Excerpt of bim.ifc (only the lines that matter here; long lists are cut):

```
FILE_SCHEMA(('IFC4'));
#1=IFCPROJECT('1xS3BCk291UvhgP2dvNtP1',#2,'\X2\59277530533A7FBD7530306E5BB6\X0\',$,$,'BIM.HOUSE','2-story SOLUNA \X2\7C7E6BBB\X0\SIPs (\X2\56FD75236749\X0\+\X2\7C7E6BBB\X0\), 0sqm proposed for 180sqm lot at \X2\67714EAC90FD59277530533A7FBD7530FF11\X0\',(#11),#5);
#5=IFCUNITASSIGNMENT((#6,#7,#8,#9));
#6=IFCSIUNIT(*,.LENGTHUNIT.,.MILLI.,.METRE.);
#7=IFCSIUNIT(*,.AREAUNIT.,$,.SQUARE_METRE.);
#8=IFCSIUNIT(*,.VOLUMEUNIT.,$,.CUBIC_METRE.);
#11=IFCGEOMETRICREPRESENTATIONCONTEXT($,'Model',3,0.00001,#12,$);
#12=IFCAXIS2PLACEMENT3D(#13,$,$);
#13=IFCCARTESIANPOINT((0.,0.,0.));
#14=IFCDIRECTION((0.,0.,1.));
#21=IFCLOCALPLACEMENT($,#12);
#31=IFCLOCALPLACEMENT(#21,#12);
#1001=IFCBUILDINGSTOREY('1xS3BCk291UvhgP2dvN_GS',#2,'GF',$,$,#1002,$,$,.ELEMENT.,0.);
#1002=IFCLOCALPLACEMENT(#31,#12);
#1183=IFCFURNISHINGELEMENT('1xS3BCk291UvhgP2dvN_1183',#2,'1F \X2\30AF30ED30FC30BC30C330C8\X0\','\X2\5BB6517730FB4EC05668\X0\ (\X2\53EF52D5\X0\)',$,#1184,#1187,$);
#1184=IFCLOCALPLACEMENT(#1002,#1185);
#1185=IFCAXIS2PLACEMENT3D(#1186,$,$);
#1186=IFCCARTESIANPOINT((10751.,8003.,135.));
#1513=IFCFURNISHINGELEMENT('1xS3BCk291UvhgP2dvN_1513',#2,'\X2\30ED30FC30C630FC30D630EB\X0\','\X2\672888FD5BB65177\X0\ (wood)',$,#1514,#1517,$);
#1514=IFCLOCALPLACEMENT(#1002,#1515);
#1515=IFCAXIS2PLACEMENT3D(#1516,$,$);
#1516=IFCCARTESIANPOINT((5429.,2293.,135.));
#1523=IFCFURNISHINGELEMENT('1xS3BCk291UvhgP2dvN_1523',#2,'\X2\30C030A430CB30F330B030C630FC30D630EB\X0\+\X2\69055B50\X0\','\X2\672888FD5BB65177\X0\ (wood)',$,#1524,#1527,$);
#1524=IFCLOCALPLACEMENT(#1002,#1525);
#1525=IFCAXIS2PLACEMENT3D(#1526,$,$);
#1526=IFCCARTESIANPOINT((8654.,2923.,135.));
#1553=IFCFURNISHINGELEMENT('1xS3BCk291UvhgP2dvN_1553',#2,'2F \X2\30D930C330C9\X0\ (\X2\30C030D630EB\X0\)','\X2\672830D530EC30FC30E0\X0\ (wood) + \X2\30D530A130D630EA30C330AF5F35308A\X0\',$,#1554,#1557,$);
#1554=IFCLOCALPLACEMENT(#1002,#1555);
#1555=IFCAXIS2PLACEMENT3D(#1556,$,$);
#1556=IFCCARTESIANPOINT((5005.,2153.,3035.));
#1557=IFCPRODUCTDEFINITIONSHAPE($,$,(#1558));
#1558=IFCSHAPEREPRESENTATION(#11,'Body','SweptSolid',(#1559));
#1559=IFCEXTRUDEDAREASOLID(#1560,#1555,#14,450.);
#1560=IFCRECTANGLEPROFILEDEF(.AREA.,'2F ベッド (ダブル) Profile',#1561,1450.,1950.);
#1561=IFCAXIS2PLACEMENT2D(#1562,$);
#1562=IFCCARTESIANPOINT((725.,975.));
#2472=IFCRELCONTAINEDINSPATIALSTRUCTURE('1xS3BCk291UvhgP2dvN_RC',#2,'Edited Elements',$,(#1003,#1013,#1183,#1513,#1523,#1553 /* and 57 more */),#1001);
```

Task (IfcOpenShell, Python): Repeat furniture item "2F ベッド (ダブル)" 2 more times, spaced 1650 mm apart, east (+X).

```python
import numpy as np
import ifcopenshell
import ifcopenshell.api.geometry
import ifcopenshell.api.root
import ifcopenshell.util.element
import ifcopenshell.util.placement
import ifcopenshell.util.unit

model = ifcopenshell.open("bim.ifc")
unit_scale = ifcopenshell.util.unit.calculate_unit_scale(model)


def reuse_history(source, copy):
    """copy_class also copies each property set's owner history, people and application; keep the originals."""
    for rel in copy.IsDefinedBy:
        if rel.is_a("IfcRelDefinesByProperties") and (history := rel.RelatingPropertyDefinition.OwnerHistory):
            rel.RelatingPropertyDefinition.OwnerHistory = source.OwnerHistory
            ifcopenshell.util.element.remove_deep2(model, history)


source = model.by_id(1553)
base = ifcopenshell.util.placement.get_local_placement(source.ObjectPlacement)
step = np.array([1.0, 0.0, 0.0]) * 1.65 / unit_scale

for i in range(1, 3):
    copy = ifcopenshell.api.root.copy_class(model, product=source)
    copy.Representation = ifcopenshell.util.element.copy_deep(
        model, source.Representation, exclude=["IfcGeometricRepresentationContext", "IfcRepresentationMap"]
    )
    reuse_history(source, copy)
    matrix = base.copy()
    matrix[:3, 3] += i * step
    print("added at", matrix[:3, 3].round(3) + 0.0)
    ifcopenshell.api.geometry.edit_object_placement(model, product=copy, matrix=matrix, is_si=False)

model.write("bim_edited.ifc")
```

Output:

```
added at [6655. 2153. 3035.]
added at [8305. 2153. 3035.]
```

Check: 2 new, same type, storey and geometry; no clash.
